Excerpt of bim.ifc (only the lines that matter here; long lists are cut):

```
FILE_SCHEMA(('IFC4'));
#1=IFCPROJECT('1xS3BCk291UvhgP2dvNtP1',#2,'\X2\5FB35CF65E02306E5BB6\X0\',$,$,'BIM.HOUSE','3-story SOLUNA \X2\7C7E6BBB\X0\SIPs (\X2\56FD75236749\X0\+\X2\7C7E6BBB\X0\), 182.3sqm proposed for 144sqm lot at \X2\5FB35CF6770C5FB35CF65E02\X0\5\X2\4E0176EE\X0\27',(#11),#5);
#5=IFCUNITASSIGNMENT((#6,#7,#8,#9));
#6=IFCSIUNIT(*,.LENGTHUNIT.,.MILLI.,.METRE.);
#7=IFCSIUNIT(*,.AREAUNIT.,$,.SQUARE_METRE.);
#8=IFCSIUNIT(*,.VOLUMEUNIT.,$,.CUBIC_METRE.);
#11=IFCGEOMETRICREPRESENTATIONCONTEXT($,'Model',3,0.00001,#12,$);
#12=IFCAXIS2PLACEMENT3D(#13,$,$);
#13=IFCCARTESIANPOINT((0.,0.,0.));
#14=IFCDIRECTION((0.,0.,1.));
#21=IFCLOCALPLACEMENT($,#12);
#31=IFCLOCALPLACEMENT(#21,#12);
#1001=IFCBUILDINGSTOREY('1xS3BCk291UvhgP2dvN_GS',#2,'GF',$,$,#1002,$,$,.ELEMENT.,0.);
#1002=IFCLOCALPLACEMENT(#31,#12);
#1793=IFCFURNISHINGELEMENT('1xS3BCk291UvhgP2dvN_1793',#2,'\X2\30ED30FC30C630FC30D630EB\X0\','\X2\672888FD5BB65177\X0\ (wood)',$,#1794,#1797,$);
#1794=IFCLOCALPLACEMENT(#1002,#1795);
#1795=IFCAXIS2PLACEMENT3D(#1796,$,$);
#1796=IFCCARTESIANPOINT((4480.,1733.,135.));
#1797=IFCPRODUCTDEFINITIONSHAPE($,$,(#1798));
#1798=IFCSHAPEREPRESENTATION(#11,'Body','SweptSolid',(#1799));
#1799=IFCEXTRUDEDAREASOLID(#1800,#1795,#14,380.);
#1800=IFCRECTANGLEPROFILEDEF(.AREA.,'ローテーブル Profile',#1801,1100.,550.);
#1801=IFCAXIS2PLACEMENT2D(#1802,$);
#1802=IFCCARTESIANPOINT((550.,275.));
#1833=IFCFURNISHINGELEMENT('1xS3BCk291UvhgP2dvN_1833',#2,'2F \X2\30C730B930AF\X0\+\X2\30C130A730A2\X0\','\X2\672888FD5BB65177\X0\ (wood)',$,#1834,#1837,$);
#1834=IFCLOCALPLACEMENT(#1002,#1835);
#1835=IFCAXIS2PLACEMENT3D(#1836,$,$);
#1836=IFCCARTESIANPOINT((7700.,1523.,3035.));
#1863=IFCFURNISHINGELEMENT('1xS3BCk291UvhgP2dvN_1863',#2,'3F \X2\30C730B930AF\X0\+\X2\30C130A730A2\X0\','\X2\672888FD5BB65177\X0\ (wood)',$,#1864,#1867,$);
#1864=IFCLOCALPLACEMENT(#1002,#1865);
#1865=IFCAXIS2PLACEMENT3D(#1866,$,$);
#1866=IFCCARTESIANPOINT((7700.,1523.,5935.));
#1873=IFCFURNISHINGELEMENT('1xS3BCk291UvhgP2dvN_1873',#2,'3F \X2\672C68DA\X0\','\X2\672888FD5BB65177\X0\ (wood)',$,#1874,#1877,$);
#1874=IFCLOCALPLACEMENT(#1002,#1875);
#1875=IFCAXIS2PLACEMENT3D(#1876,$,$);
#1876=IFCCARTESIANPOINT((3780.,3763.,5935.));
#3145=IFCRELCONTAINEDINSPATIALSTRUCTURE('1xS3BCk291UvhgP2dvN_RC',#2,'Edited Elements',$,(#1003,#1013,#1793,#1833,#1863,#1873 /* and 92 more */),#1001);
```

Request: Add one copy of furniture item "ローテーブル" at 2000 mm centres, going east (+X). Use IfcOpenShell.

```python
import numpy as np
import ifcopenshell
import ifcopenshell.api.geometry
import ifcopenshell.api.root
import ifcopenshell.util.element
import ifcopenshell.util.placement

model = ifcopenshell.open("bim.ifc")


def reuse_history(source, copy):
    """copy_class also copies each property set's owner history, people and application; keep the originals."""
    for rel in copy.IsDefinedBy:
        if rel.is_a("IfcRelDefinesByProperties") and (history := rel.RelatingPropertyDefinition.OwnerHistory):
            rel.RelatingPropertyDefinition.OwnerHistory = source.OwnerHistory
            ifcopenshell.util.element.remove_deep2(model, history)


source = model.by_guid("1xS3BCk291UvhgP2dvN_1793")
base = ifcopenshell.util.placement.get_local_placement(source.ObjectPlacement)
step = np.array([1.0, 0.0, 0.0]) * 2000.0

for i in range(1, 2):
    copy = ifcopenshell.api.root.copy_class(model, product=source)
    copy.Representation = ifcopenshell.util.element.copy_deep(
        model, source.Representation, exclude=["IfcGeometricRepresentationContext", "IfcRepresentationMap"]
    )
    reuse_history(source, copy)
    matrix = base.copy()
    matrix[:3, 3] += i * step
    print("added at", matrix[:3, 3].round(3) + 0.0)
    ifcopenshell.api.geometry.edit_object_placement(model, product=copy, matrix=matrix, is_si=False)

model.write("bim_v2.ifc")
```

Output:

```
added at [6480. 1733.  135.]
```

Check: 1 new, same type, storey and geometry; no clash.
